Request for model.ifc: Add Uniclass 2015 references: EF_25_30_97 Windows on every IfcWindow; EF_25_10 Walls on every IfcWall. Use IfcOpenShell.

First a look at what the model holds.

```python
import ifcopenshell

model = ifcopenshell.open("model.ifc")
print(model.schema)
print("classifications:", [c.Name for c in model.by_type("IfcClassification")])
for ifc_class in ("IfcDoor", "IfcRoof", "IfcStair", "IfcWall", "IfcWindow"):
    print(ifc_class, len(model.by_type(ifc_class)))
```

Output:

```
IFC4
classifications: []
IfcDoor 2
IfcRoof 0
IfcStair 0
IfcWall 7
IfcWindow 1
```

```python
import ifcopenshell
import ifcopenshell.api.classification

model = ifcopenshell.open("model.ifc")

system = ifcopenshell.api.classification.add_classification(model, classification="Uniclass 2015")

codes = {
    "IfcWindow": ("EF_25_30_97", "Windows"),
    "IfcWall": ("EF_25_10", "Walls"),
}
for ifc_class, (code, name) in codes.items():
    products = model.by_type(ifc_class)
    ifcopenshell.api.classification.add_reference(
        model, products=products, classification=system, identification=code, name=name
    )
    print(code, len(products))

model.write("model_v2.ifc")
```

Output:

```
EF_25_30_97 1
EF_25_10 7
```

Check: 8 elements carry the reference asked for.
